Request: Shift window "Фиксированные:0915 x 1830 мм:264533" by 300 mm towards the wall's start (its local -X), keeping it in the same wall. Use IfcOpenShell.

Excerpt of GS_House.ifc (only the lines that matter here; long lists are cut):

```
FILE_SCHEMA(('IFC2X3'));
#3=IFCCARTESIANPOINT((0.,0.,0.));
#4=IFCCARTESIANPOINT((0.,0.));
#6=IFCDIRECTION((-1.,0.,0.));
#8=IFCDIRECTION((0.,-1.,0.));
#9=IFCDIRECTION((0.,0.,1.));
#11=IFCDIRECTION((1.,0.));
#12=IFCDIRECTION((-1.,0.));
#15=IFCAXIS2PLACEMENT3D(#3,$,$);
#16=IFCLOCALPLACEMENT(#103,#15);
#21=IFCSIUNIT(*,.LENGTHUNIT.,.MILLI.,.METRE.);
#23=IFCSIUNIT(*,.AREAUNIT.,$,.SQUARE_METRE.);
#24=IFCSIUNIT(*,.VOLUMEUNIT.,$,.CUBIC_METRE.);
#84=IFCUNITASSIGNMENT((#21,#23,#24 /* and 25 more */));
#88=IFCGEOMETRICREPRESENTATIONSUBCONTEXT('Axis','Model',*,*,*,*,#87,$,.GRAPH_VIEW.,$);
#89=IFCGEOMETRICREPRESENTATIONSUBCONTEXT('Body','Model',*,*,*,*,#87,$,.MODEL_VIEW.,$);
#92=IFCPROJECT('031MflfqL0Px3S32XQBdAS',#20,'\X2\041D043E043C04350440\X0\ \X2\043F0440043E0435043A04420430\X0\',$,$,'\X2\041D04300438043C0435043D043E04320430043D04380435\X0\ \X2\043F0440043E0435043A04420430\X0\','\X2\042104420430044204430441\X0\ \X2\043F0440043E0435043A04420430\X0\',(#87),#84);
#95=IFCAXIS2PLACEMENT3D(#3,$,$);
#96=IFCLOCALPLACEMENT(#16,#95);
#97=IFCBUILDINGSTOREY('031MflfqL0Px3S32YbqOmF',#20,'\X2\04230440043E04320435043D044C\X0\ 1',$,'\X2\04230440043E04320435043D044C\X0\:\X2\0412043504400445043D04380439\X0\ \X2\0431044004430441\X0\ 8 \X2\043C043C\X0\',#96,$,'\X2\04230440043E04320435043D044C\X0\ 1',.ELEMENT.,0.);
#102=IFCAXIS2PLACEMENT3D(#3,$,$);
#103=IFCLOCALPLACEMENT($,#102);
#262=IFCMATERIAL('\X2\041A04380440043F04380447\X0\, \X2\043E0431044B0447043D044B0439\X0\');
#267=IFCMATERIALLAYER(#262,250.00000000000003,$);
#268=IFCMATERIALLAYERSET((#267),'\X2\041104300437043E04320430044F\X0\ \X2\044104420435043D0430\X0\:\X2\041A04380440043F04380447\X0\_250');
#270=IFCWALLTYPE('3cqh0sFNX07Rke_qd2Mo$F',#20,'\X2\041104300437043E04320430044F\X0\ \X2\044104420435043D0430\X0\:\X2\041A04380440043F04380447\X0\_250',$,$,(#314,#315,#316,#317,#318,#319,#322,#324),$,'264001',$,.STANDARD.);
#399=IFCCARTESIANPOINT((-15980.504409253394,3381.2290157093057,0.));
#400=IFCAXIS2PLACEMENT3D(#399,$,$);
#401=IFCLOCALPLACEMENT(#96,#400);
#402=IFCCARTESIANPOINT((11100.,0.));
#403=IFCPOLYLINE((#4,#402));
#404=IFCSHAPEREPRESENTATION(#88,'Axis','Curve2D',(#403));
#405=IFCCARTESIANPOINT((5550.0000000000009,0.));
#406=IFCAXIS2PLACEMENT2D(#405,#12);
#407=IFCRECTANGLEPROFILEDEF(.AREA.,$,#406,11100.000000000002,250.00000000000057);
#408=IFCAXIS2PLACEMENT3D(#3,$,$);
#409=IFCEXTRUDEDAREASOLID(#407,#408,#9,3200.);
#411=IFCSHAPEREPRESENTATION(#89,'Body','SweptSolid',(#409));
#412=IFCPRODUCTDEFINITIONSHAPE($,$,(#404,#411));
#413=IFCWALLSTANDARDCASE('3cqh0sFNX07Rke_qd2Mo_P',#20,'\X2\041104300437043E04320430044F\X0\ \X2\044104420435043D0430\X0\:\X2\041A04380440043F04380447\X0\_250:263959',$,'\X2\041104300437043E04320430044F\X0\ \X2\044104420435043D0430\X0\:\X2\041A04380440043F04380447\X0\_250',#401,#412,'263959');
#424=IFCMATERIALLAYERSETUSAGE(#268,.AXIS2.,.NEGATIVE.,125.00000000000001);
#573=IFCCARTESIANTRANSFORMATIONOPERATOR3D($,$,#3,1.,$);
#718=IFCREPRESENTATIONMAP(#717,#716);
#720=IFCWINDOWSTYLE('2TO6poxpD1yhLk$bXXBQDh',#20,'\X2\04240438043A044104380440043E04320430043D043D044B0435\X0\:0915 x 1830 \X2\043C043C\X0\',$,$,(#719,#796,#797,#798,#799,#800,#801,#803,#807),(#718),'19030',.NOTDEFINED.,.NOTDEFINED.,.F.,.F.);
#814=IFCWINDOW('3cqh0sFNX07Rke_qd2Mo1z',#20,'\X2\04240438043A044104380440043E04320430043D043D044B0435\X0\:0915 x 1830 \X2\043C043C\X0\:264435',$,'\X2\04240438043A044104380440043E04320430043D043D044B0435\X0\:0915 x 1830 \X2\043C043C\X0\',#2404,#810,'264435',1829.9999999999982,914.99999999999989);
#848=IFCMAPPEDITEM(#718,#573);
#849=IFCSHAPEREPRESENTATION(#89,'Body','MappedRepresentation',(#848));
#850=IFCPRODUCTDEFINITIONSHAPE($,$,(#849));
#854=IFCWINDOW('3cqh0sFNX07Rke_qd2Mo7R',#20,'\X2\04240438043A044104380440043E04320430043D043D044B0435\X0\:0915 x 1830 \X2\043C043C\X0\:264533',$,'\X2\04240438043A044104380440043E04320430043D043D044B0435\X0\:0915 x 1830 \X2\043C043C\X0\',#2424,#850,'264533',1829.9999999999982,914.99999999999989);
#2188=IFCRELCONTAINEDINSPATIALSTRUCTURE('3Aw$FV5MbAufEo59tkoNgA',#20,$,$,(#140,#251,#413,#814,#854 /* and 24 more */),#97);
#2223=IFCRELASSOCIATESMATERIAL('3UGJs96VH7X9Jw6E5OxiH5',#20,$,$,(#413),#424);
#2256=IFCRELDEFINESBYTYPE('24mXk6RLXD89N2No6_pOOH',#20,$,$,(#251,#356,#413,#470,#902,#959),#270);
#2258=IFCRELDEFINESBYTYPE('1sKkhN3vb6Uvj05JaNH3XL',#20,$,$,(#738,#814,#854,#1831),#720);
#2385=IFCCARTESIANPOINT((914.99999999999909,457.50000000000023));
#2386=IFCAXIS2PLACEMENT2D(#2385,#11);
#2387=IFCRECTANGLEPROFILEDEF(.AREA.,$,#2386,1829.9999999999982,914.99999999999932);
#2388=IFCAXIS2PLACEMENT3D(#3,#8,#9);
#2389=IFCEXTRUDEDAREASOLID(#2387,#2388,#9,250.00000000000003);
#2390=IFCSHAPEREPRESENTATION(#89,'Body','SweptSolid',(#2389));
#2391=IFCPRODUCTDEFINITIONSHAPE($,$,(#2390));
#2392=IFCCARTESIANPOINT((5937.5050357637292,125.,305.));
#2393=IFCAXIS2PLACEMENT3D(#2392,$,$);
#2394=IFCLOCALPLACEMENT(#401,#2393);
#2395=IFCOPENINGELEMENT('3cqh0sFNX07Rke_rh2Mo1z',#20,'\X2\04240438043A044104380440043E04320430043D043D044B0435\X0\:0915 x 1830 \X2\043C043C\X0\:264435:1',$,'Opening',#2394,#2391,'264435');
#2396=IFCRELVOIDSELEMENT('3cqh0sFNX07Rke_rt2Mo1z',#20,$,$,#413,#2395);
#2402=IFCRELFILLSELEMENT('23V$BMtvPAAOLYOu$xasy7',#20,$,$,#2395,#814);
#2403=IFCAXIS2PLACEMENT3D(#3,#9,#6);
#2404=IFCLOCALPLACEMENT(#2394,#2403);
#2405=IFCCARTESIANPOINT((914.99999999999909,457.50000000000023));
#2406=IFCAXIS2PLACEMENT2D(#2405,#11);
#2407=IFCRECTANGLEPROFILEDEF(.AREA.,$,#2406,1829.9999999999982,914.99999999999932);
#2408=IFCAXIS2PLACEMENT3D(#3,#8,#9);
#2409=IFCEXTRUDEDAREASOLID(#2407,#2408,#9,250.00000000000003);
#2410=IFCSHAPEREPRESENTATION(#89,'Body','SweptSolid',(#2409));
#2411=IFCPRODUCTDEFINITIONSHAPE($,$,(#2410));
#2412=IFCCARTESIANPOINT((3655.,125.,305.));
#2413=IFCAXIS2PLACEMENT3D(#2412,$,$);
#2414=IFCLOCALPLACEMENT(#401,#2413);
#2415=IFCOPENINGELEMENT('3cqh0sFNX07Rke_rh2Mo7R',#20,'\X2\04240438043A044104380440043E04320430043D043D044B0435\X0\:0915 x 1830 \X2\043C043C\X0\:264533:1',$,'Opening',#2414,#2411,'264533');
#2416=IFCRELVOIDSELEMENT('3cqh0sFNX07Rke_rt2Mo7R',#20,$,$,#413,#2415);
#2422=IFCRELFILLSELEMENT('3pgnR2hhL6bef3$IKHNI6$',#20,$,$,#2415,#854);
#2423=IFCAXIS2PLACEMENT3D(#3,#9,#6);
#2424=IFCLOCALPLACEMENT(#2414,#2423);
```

```python
import ifcopenshell
import ifcopenshell.api.geometry
import ifcopenshell.util.placement
import ifcopenshell.util.unit

model = ifcopenshell.open("GS_House.ifc")
unit_scale = ifcopenshell.util.unit.calculate_unit_scale(model)

window = model.by_id(854)
opening = window.FillsVoids[0].RelatingOpeningElement
wall = opening.VoidsElements[0].RelatingBuildingElement

wall_matrix = ifcopenshell.util.placement.get_local_placement(wall.ObjectPlacement)
shift = wall_matrix[:3, 0] * -0.3 / unit_scale
before = ifcopenshell.util.placement.get_local_placement(window.ObjectPlacement)[:3, 3].copy()

# The window is placed relative to its opening, so it follows when the opening moves.
matrix = ifcopenshell.util.placement.get_local_placement(opening.ObjectPlacement)
matrix[:3, 3] += shift
ifcopenshell.api.geometry.edit_object_placement(
    model, product=opening, matrix=matrix, is_si=False, should_transform_children=True
)

after = ifcopenshell.util.placement.get_local_placement(window.ObjectPlacement)[:3, 3]
print("window moved by", (after - before).round(3) + 0.0)

model.write("GS_House_edited.ifc")
```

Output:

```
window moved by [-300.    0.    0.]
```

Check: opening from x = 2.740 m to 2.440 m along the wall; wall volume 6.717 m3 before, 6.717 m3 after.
